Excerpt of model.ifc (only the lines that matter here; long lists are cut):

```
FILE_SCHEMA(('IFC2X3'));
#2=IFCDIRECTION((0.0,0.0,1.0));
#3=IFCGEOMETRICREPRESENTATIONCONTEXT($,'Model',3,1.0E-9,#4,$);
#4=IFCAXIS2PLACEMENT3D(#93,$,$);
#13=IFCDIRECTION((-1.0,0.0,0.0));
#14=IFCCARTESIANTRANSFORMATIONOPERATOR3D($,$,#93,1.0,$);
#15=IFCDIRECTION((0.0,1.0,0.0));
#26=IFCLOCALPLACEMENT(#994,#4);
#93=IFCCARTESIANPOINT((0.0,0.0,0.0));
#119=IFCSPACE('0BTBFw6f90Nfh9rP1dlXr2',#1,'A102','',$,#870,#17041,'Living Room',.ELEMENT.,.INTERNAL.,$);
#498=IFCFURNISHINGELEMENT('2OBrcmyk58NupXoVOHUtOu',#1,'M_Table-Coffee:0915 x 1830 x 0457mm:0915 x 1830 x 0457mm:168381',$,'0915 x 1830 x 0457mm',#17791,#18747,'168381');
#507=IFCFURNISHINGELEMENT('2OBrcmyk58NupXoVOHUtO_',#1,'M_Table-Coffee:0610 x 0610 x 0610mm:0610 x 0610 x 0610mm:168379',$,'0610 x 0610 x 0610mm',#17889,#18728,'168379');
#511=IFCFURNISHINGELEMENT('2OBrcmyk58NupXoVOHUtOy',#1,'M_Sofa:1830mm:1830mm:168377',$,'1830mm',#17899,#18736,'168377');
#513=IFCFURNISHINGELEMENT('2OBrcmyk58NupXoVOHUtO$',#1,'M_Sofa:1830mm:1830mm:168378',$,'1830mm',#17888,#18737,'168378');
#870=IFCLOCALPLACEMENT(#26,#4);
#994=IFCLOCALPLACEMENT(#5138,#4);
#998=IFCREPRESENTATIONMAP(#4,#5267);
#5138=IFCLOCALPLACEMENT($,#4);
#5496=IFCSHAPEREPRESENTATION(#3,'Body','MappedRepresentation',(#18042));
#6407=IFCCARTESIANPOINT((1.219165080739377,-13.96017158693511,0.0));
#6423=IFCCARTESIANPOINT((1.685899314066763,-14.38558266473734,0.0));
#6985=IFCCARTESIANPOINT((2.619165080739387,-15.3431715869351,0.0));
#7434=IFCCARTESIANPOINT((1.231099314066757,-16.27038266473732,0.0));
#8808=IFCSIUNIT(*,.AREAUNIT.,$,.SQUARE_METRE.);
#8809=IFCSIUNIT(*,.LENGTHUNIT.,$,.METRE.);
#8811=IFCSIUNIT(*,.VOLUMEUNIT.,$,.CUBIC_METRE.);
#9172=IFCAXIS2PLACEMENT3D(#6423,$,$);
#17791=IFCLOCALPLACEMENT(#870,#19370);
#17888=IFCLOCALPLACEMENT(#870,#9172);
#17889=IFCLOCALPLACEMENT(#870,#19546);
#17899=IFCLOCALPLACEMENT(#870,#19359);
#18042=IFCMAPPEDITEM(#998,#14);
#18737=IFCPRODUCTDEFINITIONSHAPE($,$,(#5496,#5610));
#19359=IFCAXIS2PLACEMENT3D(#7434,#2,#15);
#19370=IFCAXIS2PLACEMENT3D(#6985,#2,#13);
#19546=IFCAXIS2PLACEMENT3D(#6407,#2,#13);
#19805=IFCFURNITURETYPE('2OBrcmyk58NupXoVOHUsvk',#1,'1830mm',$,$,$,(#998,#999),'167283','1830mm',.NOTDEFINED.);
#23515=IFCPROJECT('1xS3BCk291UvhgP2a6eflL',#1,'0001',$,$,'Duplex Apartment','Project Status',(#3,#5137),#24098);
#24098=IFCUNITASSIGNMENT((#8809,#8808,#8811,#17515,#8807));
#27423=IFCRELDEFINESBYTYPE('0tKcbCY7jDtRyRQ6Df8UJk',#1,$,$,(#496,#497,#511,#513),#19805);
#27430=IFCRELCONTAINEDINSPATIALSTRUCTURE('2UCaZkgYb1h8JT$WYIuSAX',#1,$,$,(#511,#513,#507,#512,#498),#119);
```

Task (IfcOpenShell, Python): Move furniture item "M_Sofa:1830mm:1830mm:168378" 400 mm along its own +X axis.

```python
import ifcopenshell
import ifcopenshell.api.geometry
import ifcopenshell.util.placement
import ifcopenshell.util.unit

model = ifcopenshell.open("model.ifc")
unit_scale = ifcopenshell.util.unit.calculate_unit_scale(model)

item = model.by_guid("2OBrcmyk58NupXoVOHUtO$")
matrix = ifcopenshell.util.placement.get_local_placement(item.ObjectPlacement)
matrix[:3, 3] += matrix[:3, 0] * 0.4 / unit_scale
ifcopenshell.api.geometry.edit_object_placement(model, product=item, matrix=matrix, is_si=False)

print(ifcopenshell.util.placement.get_local_placement(item.ObjectPlacement).round(3) + 0.0)

model.write("model_v2.ifc")
```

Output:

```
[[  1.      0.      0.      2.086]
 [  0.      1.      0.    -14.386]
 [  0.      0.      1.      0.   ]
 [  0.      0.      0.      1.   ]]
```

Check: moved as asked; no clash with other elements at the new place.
